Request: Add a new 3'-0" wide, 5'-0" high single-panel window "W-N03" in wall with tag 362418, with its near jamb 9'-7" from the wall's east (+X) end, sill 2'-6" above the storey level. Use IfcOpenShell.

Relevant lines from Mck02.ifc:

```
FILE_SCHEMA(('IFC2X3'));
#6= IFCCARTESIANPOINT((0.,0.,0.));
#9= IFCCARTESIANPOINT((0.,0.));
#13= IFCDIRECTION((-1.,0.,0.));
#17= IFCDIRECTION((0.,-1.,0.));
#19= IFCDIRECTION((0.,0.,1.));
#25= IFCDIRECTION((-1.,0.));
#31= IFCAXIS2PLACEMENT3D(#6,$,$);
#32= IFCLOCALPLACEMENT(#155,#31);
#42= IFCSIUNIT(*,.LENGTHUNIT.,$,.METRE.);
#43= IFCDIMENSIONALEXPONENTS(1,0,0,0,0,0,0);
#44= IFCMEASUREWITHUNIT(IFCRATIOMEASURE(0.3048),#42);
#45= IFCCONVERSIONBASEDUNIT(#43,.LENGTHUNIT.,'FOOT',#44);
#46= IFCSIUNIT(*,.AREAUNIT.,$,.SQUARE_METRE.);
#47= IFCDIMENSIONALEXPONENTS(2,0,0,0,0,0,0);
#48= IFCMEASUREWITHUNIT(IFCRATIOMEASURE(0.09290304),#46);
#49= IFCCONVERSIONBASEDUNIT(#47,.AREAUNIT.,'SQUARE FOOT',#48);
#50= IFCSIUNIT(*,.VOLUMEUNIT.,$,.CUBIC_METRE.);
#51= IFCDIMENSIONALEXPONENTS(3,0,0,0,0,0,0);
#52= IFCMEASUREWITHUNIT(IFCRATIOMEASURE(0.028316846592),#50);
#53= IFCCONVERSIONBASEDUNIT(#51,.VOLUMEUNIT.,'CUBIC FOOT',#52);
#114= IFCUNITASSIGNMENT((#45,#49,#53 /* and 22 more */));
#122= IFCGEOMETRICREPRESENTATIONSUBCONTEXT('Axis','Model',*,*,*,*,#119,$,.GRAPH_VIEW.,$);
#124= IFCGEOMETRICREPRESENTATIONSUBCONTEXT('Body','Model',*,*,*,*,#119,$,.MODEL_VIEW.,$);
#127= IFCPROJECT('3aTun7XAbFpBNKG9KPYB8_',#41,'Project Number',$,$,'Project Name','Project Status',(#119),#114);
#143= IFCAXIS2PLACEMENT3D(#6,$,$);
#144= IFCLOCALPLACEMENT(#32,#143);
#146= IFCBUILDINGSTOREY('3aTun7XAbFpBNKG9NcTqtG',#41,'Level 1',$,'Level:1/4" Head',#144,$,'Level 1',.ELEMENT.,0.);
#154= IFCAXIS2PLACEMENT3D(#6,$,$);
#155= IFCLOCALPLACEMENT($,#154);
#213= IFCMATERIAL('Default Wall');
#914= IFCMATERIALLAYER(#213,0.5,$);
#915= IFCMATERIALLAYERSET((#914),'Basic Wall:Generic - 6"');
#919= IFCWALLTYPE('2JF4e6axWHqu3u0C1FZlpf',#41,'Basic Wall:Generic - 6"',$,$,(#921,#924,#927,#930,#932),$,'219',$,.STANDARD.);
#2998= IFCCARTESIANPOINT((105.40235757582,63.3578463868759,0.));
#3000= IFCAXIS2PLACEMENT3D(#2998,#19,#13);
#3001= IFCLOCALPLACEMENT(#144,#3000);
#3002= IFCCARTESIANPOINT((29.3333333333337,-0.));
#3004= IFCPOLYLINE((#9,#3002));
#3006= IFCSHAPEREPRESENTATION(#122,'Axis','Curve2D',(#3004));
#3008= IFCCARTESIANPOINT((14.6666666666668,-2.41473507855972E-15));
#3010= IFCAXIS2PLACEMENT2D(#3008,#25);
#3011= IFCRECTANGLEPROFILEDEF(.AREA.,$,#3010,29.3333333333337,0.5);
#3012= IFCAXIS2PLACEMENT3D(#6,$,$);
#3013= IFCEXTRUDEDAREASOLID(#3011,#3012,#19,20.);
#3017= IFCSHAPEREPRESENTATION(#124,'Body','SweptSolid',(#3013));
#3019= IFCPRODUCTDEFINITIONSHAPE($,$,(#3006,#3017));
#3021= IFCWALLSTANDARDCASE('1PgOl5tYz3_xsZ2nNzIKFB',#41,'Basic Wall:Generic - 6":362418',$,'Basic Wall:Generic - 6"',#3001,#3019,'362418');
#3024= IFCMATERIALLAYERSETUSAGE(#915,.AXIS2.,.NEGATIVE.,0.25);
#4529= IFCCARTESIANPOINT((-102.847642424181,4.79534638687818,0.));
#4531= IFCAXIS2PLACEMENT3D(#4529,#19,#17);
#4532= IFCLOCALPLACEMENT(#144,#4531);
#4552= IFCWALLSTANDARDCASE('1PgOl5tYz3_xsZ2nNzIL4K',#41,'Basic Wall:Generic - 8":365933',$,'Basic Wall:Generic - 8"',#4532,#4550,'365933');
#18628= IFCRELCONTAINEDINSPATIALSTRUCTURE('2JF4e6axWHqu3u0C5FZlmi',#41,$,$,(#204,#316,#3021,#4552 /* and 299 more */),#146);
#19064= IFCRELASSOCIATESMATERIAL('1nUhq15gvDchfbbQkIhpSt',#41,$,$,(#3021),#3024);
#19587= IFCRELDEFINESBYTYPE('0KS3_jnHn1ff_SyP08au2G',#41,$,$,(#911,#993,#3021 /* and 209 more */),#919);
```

```python
import numpy as np
import ifcopenshell
import ifcopenshell.api.feature
import ifcopenshell.api.geometry
import ifcopenshell.api.root
import ifcopenshell.api.spatial
import ifcopenshell.api.type
import ifcopenshell.geom
import ifcopenshell.util.element
import ifcopenshell.util.placement
import ifcopenshell.util.representation
import ifcopenshell.util.shape
import ifcopenshell.util.unit

model = ifcopenshell.open("Mck02.ifc")
unit_scale = ifcopenshell.util.unit.calculate_unit_scale(model)
settings = ifcopenshell.geom.settings()


def volume(element):
    """Net volume in cubic metres, openings subtracted."""
    shape = ifcopenshell.geom.create_shape(settings, element)
    return ifcopenshell.util.shape.get_volume(shape.geometry)


wall = model.by_guid("1PgOl5tYz3_xsZ2nNzIKFB")
storey = ifcopenshell.util.element.get_container(wall, ifc_class="IfcBuildingStorey")
context = ifcopenshell.util.representation.get_context(model, "Model", "Body", "MODEL_VIEW")
before = volume(wall)

width, height, from_end, sill = 0.9144, 1.524, 2.921, 0.762  # metres

# The wall runs along its own X axis, and the end named is its -X end.
wall_shape = ifcopenshell.geom.create_shape(settings, wall)
x, y, z = ifcopenshell.util.shape.get_vertices(wall_shape.geometry).T
start = x.min() + from_end
face, thickness = float(y.min()), float(y.max() - y.min())
wall_matrix = ifcopenshell.util.placement.get_local_placement(wall.ObjectPlacement)
level = ifcopenshell.util.placement.get_local_placement(storey.ObjectPlacement)[2, 3]


def in_wall(x, y):
    """Placement at x, y metres in the wall's axes, at sill height."""
    matrix = wall_matrix.copy()
    matrix[:, 3] = wall_matrix @ np.array([x / unit_scale, y / unit_scale, 0.0, 1.0])
    matrix[2, 3] = level + sill / unit_scale
    return matrix


# Opening: a box that overshoots both wall faces by 50 mm.
opening = ifcopenshell.api.root.create_entity(model, ifc_class="IfcOpeningElement")
box = ifcopenshell.api.geometry.add_wall_representation(
    model, context=context, length=width, height=height, thickness=thickness + 0.1
)
ifcopenshell.api.geometry.assign_representation(model, product=opening, representation=box)
ifcopenshell.api.geometry.edit_object_placement(model, product=opening, matrix=in_wall(start, face - 0.05), is_si=False)
ifcopenshell.api.feature.add_feature(model, feature=opening, element=wall)

window = ifcopenshell.api.root.create_entity(model, ifc_class="IfcWindow", name="W-N03")
window.OverallWidth, window.OverallHeight = width / unit_scale, height / unit_scale
body = ifcopenshell.api.geometry.add_window_representation(
    model,
    context=context,
    overall_width=window.OverallWidth,
    overall_height=window.OverallHeight,
    partition_type="SINGLE_PANEL",
)
ifcopenshell.api.geometry.assign_representation(model, product=window, representation=body)
ifcopenshell.api.spatial.assign_container(model, products=[window], relating_structure=storey)
fills = ifcopenshell.api.feature.add_filling(model, opening=opening, element=window)
fills.OwnerHistory = window.OwnerHistory  # required in IFC2X3

# IFC2X3 keeps the operation on the window style.
style = ifcopenshell.api.root.create_entity(model, ifc_class="IfcWindowStyle", name="W-N03")
style.OperationType, style.ConstructionType = "SINGLE_PANEL", "NOTDEFINED"
style.ParameterTakesPrecedence = style.Sizeable = False
ifcopenshell.api.type.assign_type(model, related_objects=[window], relating_type=style)

# Centre the window in the wall's thickness.
ifcopenshell.api.geometry.edit_object_placement(model, product=window, matrix=in_wall(start, face), is_si=False)
window_shape = ifcopenshell.geom.create_shape(settings, window)
depth = ifcopenshell.util.shape.get_vertices(window_shape.geometry)[:, 1]
offset = face + thickness / 2 - (depth.min() + depth.max()) / 2
ifcopenshell.api.geometry.edit_object_placement(model, product=window, matrix=in_wall(start, offset), is_si=False)

after = volume(wall)

print(f"wall volume {before:.3f} -> {after:.3f} m3")

model.write("Mck02_updated.ifc")
```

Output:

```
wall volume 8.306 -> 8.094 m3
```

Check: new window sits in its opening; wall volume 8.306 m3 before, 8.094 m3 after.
